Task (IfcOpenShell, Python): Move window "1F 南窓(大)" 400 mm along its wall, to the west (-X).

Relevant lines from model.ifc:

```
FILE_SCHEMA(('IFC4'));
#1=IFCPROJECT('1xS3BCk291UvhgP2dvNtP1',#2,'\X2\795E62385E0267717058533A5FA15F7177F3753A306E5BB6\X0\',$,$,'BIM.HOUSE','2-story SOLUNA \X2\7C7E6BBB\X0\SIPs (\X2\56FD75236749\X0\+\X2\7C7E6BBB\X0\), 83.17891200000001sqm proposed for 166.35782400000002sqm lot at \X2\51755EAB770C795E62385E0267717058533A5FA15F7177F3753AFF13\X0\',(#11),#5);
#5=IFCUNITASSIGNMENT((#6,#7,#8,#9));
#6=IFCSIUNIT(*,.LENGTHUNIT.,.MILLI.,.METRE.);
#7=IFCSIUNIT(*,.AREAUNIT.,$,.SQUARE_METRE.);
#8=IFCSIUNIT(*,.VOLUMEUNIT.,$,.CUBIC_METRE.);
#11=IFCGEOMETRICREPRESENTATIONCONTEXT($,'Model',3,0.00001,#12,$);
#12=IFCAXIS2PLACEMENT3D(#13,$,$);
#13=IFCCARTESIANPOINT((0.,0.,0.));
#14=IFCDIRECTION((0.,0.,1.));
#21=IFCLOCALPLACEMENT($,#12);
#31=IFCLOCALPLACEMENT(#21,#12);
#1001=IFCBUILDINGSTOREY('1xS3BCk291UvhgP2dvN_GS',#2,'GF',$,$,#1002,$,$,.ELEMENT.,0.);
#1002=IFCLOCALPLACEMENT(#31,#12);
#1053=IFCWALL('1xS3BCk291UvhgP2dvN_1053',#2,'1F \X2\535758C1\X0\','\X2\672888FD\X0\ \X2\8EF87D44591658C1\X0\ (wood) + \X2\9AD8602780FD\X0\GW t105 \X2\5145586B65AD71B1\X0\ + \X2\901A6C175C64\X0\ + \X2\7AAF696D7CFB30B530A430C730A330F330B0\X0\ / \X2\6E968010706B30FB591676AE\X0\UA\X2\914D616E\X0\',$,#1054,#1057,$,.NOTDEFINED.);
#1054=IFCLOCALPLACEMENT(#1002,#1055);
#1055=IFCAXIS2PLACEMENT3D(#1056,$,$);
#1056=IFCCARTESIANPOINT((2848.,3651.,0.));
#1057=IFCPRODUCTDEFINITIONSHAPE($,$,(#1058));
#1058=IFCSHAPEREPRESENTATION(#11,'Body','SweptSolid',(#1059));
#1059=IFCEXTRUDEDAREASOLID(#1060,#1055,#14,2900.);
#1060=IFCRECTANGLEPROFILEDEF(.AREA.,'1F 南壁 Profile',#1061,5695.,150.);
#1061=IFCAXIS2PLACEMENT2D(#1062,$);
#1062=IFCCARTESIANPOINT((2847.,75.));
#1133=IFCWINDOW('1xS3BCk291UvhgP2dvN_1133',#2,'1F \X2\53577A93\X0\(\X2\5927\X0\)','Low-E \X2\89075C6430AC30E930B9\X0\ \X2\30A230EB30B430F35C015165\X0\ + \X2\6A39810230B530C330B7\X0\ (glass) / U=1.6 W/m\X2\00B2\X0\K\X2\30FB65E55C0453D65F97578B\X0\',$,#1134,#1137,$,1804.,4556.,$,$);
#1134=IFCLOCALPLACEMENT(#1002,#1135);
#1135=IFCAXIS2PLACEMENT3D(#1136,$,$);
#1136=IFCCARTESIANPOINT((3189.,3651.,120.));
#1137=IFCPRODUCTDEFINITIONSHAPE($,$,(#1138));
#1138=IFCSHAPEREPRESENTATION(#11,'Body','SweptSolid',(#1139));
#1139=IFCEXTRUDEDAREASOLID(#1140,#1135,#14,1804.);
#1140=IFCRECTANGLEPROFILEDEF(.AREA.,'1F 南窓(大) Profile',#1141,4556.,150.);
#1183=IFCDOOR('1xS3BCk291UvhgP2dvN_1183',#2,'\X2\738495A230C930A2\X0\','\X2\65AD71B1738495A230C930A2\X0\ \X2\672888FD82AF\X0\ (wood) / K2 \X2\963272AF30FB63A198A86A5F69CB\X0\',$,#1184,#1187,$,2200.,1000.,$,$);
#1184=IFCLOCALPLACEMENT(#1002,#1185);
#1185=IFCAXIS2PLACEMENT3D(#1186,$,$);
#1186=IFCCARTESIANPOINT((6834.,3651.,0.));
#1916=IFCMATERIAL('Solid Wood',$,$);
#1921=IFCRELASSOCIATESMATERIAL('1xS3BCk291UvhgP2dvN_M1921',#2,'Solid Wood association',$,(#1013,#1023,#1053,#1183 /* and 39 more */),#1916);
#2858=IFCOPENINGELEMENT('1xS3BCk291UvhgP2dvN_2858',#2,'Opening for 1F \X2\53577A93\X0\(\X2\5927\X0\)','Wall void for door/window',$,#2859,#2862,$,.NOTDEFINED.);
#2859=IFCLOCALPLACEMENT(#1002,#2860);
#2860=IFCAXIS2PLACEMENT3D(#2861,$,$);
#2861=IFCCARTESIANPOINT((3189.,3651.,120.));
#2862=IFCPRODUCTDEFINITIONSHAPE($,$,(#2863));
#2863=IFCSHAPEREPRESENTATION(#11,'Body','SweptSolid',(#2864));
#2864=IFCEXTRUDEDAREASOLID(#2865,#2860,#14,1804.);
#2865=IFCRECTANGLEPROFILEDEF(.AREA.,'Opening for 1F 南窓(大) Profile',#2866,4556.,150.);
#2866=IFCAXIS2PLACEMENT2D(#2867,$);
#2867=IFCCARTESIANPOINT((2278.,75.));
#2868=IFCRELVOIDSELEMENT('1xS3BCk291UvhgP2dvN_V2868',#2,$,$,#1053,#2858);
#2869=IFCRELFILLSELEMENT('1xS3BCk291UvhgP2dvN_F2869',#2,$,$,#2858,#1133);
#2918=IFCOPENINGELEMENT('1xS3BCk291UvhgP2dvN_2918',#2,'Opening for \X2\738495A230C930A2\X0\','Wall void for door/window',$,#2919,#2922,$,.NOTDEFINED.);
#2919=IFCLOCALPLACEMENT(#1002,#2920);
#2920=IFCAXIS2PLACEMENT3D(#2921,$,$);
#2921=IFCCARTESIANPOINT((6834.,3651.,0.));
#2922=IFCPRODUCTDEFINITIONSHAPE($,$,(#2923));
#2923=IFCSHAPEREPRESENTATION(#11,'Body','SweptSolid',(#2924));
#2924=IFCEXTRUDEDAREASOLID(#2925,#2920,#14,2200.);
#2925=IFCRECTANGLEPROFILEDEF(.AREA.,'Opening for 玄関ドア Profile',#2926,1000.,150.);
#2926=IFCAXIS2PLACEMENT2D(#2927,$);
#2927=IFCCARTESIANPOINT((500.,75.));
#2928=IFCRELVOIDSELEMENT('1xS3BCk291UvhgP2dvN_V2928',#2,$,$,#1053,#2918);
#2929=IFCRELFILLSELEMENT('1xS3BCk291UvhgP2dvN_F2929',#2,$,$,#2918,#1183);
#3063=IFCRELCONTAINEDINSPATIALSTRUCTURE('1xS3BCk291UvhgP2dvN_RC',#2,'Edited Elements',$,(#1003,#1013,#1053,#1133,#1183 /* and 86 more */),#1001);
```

```python
import ifcopenshell
import ifcopenshell.api.geometry
import ifcopenshell.util.placement

model = ifcopenshell.open("model.ifc")

window = model.by_guid("1xS3BCk291UvhgP2dvN_1133")
opening = window.FillsVoids[0].RelatingOpeningElement
wall = opening.VoidsElements[0].RelatingBuildingElement

wall_matrix = ifcopenshell.util.placement.get_local_placement(wall.ObjectPlacement)
shift = wall_matrix[:3, 0] * -400.0
before = ifcopenshell.util.placement.get_local_placement(window.ObjectPlacement)[:3, 3].copy()

# The window is not placed relative to its opening, so move both.
for product in (opening, window):
    matrix = ifcopenshell.util.placement.get_local_placement(product.ObjectPlacement)
    matrix[:3, 3] += shift
    ifcopenshell.api.geometry.edit_object_placement(model, product=product, matrix=matrix, is_si=False)

after = ifcopenshell.util.placement.get_local_placement(window.ObjectPlacement)[:3, 3]
print("window moved by", (after - before).round(3) + 0.0)

model.write("model_edited.ifc")
```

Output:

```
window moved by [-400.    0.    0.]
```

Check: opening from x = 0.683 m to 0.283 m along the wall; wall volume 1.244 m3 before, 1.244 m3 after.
